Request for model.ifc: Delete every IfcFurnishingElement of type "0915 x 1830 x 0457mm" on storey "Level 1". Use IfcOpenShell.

First a look at what the model holds.

```python
import ifcopenshell
import ifcopenshell.util.element

model = ifcopenshell.open("model.ifc")
print(model.schema)
storey = next(s for s in model.by_type("IfcBuildingStorey") if s.Name == "Level 1")
furniture = [e for e in ifcopenshell.util.element.get_decomposition(storey) if e.is_a("IfcFurnishingElement")]
seen = {}
for e in furniture:
    element_type = ifcopenshell.util.element.get_type(e)
    name = element_type.Name if element_type not in (None, e) else None
    seen[name] = seen.get(name, 0) + 1
for name, count in sorted(seen.items(), key=str):
    print(count, "x", name)
```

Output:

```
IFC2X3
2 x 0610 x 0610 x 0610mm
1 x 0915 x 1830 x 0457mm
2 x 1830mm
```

```python
import ifcopenshell
import ifcopenshell.api.root
import ifcopenshell.util.element

model = ifcopenshell.open("model.ifc")

storey = next(s for s in model.by_type("IfcBuildingStorey") if s.Name == "Level 1")
furniture = [e for e in ifcopenshell.util.element.get_decomposition(storey) if e.is_a("IfcFurnishingElement")]
targets = [e for e in furniture if (t := ifcopenshell.util.element.get_type(e)) not in (None, e) and t.Name == "0915 x 1830 x 0457mm"]

for e in targets:
    ifcopenshell.api.root.remove_product(model, product=e)
print(len(targets), "removed")

model.write("model_rev.ifc")
```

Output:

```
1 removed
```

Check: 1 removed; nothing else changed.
